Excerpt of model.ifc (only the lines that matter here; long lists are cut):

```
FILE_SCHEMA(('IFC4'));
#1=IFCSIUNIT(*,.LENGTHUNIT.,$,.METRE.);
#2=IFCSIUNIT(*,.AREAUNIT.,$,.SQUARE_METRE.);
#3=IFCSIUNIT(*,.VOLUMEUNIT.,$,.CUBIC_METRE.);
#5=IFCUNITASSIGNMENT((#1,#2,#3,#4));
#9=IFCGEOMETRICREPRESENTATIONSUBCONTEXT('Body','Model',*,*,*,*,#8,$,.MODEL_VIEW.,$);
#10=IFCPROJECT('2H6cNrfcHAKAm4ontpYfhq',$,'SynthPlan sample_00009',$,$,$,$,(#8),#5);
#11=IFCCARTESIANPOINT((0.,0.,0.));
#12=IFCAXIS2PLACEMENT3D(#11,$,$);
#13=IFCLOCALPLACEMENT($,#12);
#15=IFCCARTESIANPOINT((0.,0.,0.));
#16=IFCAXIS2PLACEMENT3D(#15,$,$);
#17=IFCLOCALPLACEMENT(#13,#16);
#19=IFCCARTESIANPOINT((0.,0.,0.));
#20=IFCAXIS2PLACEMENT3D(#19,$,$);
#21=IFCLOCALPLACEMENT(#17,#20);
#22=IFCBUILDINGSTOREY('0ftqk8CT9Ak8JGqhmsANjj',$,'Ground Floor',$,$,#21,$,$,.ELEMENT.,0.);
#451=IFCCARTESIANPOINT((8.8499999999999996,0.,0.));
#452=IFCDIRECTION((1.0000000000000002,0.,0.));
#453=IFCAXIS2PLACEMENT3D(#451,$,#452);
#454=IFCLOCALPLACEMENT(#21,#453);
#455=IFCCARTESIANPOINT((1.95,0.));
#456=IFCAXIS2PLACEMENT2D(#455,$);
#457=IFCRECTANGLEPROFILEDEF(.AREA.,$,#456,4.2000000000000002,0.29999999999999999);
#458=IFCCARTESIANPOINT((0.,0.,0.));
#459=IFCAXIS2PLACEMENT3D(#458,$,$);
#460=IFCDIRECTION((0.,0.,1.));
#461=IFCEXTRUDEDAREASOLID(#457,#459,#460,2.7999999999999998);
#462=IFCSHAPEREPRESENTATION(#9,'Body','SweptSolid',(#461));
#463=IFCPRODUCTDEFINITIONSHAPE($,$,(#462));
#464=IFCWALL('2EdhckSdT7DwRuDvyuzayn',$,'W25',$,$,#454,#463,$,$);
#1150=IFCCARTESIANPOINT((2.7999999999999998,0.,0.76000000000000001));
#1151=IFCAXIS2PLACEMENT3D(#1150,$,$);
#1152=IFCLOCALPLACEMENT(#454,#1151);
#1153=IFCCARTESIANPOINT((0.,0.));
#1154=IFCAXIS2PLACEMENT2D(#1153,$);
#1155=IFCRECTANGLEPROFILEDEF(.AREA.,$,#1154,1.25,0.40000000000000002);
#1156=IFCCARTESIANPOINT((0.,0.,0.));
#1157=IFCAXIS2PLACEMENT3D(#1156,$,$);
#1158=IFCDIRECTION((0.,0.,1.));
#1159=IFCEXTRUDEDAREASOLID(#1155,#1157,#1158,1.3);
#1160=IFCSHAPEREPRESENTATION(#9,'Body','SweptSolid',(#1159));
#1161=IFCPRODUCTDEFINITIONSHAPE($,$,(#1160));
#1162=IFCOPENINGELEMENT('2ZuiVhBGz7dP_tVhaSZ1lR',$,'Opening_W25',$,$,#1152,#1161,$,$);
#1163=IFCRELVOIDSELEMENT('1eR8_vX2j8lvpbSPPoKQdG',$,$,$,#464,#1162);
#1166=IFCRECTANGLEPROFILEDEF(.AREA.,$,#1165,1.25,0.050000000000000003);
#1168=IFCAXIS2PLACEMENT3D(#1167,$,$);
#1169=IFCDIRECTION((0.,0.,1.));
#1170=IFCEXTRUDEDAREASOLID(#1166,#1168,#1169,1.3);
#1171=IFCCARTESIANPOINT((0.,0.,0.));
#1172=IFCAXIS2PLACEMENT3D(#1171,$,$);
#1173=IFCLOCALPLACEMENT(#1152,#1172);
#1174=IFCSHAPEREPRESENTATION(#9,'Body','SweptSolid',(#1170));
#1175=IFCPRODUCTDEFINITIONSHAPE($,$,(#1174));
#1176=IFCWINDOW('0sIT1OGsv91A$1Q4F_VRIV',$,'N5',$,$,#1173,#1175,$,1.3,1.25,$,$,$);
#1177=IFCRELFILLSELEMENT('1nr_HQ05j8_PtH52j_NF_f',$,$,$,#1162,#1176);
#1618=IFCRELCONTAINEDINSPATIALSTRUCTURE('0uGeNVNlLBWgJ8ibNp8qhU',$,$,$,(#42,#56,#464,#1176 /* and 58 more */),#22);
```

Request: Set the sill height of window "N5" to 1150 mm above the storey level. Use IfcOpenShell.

```python
import numpy as np
import ifcopenshell
import ifcopenshell.api.geometry
import ifcopenshell.geom
import ifcopenshell.util.element
import ifcopenshell.util.placement
import ifcopenshell.util.shape
import ifcopenshell.util.unit

model = ifcopenshell.open("model.ifc")
unit_scale = ifcopenshell.util.unit.calculate_unit_scale(model)

window = model.by_guid("0sIT1OGsv91A$1Q4F_VRIV")
opening = window.FillsVoids[0].RelatingOpeningElement
storey = ifcopenshell.util.element.get_container(window, ifc_class="IfcBuildingStorey")
level = ifcopenshell.util.placement.get_local_placement(storey.ObjectPlacement)[2, 3]

# The opening's origin need not be at the sill, so measure its lowest point.
shape = ifcopenshell.geom.create_shape(ifcopenshell.geom.settings(), opening)
bottom = ifcopenshell.util.shape.get_shape_bottom_elevation(shape, shape.geometry) / unit_scale
dz = level + 1.15 / unit_scale - bottom

shift = np.array([0.0, 0.0, dz])
# The window is placed relative to its opening, so it follows when the opening moves.
matrix = ifcopenshell.util.placement.get_local_placement(opening.ObjectPlacement)
matrix[:3, 3] += shift
ifcopenshell.api.geometry.edit_object_placement(
    model, product=opening, matrix=matrix, is_si=False, should_transform_children=True
)

print(f"moved by {dz * unit_scale:+.3f} m")

model.write("model_updated.ifc")
```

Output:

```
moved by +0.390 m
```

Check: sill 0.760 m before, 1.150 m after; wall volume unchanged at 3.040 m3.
